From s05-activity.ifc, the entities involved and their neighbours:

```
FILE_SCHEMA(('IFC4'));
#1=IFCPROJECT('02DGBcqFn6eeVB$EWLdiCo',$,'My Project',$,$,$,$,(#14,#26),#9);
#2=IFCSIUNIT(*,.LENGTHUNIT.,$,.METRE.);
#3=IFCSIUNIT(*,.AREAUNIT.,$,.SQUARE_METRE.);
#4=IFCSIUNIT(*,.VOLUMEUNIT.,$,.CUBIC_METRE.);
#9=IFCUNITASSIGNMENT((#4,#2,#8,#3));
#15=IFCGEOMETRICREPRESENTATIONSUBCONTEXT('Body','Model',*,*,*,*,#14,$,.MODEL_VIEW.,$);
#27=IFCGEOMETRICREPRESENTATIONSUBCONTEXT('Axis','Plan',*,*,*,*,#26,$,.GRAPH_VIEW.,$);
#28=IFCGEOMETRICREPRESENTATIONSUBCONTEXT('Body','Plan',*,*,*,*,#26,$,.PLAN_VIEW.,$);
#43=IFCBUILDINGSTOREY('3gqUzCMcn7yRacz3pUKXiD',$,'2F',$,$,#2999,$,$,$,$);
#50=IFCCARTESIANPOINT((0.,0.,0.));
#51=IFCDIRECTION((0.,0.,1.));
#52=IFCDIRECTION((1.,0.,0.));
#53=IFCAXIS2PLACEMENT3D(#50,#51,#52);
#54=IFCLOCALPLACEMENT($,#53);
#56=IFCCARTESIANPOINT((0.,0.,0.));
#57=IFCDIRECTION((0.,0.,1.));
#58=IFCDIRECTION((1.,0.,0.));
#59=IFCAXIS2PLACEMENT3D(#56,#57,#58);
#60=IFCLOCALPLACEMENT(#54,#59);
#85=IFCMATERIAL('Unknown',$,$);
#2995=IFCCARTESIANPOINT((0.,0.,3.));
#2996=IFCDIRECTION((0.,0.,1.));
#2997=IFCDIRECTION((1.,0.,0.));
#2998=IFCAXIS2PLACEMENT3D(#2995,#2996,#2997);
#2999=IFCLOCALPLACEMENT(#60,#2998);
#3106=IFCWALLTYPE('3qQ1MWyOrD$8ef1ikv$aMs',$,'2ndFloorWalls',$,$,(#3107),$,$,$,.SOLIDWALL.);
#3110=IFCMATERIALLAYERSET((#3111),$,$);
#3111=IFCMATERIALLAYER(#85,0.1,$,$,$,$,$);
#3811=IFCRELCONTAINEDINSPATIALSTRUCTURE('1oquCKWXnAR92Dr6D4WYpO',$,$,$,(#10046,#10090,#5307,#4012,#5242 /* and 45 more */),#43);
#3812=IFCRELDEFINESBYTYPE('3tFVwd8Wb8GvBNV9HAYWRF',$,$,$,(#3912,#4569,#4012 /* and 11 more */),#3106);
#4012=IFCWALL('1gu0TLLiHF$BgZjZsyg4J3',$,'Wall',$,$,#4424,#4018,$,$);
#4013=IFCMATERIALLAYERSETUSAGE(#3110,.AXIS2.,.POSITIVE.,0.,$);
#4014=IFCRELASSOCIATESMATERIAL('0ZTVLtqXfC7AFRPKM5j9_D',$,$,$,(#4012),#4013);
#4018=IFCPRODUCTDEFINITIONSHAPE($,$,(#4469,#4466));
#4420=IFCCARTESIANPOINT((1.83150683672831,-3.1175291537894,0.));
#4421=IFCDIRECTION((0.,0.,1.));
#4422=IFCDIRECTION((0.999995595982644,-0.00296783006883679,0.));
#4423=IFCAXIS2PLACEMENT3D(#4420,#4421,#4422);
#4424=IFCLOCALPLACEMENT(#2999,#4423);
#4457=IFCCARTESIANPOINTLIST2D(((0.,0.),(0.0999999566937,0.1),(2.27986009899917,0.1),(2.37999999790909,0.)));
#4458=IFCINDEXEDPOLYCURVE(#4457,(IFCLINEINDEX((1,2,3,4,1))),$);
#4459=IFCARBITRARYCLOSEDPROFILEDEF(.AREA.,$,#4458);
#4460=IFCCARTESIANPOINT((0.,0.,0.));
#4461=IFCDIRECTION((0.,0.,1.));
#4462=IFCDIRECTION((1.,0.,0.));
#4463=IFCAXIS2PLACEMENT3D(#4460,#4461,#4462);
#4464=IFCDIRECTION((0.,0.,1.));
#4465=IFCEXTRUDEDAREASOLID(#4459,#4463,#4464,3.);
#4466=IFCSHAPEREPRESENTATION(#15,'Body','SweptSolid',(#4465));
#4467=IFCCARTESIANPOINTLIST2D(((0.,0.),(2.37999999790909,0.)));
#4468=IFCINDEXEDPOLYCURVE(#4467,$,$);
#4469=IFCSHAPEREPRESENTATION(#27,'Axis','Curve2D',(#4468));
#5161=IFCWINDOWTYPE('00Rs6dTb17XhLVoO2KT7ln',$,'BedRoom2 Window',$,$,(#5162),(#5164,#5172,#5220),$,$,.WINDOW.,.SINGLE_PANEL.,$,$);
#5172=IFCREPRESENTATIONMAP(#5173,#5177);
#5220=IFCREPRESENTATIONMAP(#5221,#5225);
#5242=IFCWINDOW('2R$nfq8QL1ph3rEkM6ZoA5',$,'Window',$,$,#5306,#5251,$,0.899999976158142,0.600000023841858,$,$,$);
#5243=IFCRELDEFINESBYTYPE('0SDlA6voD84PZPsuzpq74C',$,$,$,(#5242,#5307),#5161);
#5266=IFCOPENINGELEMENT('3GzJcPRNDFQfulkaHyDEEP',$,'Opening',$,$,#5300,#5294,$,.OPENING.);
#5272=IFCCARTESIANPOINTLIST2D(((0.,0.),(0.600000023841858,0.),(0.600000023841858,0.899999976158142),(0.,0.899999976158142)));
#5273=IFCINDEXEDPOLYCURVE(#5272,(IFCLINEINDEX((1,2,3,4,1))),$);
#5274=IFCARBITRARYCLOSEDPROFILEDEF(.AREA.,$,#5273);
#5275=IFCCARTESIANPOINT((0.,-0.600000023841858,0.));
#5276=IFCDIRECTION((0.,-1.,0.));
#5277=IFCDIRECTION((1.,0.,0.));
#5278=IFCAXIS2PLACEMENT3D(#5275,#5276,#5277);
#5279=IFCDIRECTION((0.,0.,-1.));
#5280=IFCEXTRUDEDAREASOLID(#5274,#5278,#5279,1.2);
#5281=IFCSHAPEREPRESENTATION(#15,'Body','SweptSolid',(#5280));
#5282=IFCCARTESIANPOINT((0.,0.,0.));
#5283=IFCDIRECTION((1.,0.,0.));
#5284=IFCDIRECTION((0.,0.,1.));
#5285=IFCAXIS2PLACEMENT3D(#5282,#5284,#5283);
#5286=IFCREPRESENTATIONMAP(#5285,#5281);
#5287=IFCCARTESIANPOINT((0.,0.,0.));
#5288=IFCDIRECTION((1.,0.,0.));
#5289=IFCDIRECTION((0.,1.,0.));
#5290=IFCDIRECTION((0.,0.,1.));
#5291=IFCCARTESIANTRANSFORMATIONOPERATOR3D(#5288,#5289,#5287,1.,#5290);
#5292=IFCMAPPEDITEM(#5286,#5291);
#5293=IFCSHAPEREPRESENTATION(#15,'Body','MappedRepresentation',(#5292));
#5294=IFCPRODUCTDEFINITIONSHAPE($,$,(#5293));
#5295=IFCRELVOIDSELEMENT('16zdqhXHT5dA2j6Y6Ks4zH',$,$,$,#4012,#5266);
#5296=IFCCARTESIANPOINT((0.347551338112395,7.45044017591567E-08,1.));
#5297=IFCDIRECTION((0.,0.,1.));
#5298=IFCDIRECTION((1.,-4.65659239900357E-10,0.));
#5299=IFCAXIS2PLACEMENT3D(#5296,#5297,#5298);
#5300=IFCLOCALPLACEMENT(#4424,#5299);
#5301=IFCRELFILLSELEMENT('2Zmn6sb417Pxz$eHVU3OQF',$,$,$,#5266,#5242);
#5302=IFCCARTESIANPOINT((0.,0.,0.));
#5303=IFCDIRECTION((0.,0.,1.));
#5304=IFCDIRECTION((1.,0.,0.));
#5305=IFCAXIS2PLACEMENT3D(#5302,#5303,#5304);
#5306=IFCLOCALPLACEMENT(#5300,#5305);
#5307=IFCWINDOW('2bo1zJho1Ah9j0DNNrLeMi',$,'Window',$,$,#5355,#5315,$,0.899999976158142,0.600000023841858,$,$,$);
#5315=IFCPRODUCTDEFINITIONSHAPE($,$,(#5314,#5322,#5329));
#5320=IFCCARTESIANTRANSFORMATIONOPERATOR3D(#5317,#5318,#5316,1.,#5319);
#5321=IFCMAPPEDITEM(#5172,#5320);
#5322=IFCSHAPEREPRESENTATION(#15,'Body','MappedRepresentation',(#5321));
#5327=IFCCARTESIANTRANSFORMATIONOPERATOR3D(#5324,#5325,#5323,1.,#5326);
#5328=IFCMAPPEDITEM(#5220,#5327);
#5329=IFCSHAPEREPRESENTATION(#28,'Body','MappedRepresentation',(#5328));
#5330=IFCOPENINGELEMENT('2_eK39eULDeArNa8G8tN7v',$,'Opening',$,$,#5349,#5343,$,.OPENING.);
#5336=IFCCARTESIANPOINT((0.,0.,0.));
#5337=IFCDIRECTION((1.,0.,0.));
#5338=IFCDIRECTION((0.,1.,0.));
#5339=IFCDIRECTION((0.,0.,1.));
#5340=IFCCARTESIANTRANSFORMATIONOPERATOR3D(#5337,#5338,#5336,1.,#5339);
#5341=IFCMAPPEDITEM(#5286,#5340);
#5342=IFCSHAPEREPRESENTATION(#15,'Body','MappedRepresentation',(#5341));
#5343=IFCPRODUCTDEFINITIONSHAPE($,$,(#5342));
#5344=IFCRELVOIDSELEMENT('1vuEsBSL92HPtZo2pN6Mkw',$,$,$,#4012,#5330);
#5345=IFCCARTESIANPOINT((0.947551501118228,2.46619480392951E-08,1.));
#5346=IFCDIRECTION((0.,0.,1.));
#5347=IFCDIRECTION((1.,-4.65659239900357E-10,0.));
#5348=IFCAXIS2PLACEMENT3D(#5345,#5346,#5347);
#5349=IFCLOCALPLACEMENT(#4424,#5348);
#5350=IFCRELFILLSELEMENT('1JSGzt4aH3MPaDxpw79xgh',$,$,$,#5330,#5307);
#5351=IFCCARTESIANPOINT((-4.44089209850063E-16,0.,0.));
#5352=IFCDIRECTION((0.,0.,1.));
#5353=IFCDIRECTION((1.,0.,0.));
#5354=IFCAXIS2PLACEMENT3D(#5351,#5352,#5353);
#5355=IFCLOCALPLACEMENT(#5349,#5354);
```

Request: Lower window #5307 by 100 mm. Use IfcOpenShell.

```python
import numpy as np
import ifcopenshell
import ifcopenshell.api.geometry
import ifcopenshell.util.placement
import ifcopenshell.util.unit

model = ifcopenshell.open("s05-activity.ifc")
unit_scale = ifcopenshell.util.unit.calculate_unit_scale(model)

window = model.by_guid("2bo1zJho1Ah9j0DNNrLeMi")
opening = window.FillsVoids[0].RelatingOpeningElement
dz = -0.1

shift = np.array([0.0, 0.0, dz])
# The window is placed relative to its opening, so it follows when the opening moves.
matrix = ifcopenshell.util.placement.get_local_placement(opening.ObjectPlacement)
matrix[:3, 3] += shift
ifcopenshell.api.geometry.edit_object_placement(
    model, product=opening, matrix=matrix, is_si=False, should_transform_children=True
)

print(f"moved by {dz * unit_scale:+.3f} m")

model.write("s05-activity_updated.ifc")
```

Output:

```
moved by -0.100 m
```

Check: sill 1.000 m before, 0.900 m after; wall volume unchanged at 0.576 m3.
